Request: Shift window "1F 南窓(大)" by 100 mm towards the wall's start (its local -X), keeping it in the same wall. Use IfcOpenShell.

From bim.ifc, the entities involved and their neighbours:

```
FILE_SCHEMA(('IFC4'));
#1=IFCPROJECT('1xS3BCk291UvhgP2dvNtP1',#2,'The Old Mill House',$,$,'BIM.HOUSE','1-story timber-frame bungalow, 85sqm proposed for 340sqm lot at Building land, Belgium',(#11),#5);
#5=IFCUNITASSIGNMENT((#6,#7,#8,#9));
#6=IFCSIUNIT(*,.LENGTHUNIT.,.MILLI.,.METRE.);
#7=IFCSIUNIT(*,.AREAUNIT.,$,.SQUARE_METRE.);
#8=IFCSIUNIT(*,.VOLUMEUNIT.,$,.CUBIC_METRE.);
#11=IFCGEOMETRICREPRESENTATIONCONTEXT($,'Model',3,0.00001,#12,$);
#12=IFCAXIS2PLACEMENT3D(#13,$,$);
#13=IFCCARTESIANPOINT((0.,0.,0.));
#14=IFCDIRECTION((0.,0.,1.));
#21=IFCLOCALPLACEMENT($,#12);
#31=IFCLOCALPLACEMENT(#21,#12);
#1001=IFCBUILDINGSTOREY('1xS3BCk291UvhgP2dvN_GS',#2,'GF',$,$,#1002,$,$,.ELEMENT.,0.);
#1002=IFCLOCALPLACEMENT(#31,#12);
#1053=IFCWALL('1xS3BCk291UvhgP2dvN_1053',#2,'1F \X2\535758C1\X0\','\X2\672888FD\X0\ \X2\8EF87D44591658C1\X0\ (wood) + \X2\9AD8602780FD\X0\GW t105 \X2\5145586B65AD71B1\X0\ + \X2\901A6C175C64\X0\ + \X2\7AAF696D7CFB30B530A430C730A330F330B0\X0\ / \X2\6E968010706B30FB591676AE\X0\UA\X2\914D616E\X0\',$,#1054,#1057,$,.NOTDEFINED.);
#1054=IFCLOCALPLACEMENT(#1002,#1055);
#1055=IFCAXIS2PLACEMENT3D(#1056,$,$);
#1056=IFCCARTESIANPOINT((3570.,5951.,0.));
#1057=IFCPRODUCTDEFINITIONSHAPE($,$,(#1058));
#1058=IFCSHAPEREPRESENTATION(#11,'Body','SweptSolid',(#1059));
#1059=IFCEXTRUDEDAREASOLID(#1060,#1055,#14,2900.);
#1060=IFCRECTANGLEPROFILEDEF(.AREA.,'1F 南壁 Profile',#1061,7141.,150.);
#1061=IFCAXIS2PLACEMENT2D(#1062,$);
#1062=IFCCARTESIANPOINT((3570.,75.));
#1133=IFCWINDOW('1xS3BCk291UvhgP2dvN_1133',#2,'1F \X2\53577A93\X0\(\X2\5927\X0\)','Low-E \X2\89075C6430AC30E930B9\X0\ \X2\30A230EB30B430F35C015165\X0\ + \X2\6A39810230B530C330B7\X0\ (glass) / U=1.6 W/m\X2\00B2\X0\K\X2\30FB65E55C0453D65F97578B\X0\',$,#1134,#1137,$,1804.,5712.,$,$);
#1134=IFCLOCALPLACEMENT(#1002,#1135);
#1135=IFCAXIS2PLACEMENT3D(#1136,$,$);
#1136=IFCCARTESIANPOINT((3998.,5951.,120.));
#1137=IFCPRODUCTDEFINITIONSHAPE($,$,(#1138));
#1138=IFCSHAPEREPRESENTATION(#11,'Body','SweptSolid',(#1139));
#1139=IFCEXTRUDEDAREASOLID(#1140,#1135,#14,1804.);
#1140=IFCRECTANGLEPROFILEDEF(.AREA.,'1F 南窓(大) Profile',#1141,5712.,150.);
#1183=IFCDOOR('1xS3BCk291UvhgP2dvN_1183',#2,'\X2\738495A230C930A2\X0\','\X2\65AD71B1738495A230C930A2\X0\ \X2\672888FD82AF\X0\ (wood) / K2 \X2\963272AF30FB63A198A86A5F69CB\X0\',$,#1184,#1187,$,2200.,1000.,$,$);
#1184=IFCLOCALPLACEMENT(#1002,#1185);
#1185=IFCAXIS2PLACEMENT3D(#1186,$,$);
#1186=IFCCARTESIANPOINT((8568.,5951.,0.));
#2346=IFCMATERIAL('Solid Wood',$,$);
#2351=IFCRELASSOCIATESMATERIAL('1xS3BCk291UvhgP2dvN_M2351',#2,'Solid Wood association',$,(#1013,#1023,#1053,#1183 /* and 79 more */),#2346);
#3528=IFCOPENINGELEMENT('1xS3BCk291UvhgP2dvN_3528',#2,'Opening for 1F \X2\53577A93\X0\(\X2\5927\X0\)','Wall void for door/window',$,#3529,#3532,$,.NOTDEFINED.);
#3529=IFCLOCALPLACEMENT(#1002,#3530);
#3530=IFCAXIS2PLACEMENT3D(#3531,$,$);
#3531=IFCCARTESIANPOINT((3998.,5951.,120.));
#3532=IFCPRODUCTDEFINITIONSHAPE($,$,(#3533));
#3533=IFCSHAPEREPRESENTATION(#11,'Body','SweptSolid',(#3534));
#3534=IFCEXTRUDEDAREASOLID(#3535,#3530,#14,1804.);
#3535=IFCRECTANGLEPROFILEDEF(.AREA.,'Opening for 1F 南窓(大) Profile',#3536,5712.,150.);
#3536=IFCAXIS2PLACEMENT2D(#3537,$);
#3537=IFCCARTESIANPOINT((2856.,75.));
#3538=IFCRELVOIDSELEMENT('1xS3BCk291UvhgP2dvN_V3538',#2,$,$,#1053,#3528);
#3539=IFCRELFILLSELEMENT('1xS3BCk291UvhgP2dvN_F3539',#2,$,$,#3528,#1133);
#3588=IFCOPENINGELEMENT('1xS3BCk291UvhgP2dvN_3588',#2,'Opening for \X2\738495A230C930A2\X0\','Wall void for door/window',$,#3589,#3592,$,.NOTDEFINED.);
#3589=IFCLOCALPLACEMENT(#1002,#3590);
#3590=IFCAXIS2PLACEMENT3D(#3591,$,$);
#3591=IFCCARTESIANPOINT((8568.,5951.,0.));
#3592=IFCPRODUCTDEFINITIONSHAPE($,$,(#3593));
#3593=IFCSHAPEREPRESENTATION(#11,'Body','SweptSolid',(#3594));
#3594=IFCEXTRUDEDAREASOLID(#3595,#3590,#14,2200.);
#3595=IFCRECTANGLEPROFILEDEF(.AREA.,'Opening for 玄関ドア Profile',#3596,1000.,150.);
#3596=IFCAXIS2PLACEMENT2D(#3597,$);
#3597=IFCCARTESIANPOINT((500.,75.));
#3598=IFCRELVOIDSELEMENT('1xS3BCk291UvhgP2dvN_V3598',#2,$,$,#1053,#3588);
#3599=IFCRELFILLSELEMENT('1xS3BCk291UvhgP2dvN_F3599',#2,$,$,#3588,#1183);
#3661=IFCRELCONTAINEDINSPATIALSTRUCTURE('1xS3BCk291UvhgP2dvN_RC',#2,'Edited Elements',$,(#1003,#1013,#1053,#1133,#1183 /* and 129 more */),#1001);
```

```python
import ifcopenshell
import ifcopenshell.api.geometry
import ifcopenshell.util.placement
import ifcopenshell.util.unit

model = ifcopenshell.open("bim.ifc")
unit_scale = ifcopenshell.util.unit.calculate_unit_scale(model)

window = model.by_guid("1xS3BCk291UvhgP2dvN_1133")
opening = window.FillsVoids[0].RelatingOpeningElement
wall = opening.VoidsElements[0].RelatingBuildingElement

wall_matrix = ifcopenshell.util.placement.get_local_placement(wall.ObjectPlacement)
shift = wall_matrix[:3, 0] * -0.1 / unit_scale
before = ifcopenshell.util.placement.get_local_placement(window.ObjectPlacement)[:3, 3].copy()

# The window is not placed relative to its opening, so move both.
for product in (opening, window):
    matrix = ifcopenshell.util.placement.get_local_placement(product.ObjectPlacement)
    matrix[:3, 3] += shift
    ifcopenshell.api.geometry.edit_object_placement(model, product=product, matrix=matrix, is_si=False)

after = ifcopenshell.util.placement.get_local_placement(window.ObjectPlacement)[:3, 3]
print("window moved by", (after - before).round(3) + 0.0)

model.write("bim-out.ifc")
```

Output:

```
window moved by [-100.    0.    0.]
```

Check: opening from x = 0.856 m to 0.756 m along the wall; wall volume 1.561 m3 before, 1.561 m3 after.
